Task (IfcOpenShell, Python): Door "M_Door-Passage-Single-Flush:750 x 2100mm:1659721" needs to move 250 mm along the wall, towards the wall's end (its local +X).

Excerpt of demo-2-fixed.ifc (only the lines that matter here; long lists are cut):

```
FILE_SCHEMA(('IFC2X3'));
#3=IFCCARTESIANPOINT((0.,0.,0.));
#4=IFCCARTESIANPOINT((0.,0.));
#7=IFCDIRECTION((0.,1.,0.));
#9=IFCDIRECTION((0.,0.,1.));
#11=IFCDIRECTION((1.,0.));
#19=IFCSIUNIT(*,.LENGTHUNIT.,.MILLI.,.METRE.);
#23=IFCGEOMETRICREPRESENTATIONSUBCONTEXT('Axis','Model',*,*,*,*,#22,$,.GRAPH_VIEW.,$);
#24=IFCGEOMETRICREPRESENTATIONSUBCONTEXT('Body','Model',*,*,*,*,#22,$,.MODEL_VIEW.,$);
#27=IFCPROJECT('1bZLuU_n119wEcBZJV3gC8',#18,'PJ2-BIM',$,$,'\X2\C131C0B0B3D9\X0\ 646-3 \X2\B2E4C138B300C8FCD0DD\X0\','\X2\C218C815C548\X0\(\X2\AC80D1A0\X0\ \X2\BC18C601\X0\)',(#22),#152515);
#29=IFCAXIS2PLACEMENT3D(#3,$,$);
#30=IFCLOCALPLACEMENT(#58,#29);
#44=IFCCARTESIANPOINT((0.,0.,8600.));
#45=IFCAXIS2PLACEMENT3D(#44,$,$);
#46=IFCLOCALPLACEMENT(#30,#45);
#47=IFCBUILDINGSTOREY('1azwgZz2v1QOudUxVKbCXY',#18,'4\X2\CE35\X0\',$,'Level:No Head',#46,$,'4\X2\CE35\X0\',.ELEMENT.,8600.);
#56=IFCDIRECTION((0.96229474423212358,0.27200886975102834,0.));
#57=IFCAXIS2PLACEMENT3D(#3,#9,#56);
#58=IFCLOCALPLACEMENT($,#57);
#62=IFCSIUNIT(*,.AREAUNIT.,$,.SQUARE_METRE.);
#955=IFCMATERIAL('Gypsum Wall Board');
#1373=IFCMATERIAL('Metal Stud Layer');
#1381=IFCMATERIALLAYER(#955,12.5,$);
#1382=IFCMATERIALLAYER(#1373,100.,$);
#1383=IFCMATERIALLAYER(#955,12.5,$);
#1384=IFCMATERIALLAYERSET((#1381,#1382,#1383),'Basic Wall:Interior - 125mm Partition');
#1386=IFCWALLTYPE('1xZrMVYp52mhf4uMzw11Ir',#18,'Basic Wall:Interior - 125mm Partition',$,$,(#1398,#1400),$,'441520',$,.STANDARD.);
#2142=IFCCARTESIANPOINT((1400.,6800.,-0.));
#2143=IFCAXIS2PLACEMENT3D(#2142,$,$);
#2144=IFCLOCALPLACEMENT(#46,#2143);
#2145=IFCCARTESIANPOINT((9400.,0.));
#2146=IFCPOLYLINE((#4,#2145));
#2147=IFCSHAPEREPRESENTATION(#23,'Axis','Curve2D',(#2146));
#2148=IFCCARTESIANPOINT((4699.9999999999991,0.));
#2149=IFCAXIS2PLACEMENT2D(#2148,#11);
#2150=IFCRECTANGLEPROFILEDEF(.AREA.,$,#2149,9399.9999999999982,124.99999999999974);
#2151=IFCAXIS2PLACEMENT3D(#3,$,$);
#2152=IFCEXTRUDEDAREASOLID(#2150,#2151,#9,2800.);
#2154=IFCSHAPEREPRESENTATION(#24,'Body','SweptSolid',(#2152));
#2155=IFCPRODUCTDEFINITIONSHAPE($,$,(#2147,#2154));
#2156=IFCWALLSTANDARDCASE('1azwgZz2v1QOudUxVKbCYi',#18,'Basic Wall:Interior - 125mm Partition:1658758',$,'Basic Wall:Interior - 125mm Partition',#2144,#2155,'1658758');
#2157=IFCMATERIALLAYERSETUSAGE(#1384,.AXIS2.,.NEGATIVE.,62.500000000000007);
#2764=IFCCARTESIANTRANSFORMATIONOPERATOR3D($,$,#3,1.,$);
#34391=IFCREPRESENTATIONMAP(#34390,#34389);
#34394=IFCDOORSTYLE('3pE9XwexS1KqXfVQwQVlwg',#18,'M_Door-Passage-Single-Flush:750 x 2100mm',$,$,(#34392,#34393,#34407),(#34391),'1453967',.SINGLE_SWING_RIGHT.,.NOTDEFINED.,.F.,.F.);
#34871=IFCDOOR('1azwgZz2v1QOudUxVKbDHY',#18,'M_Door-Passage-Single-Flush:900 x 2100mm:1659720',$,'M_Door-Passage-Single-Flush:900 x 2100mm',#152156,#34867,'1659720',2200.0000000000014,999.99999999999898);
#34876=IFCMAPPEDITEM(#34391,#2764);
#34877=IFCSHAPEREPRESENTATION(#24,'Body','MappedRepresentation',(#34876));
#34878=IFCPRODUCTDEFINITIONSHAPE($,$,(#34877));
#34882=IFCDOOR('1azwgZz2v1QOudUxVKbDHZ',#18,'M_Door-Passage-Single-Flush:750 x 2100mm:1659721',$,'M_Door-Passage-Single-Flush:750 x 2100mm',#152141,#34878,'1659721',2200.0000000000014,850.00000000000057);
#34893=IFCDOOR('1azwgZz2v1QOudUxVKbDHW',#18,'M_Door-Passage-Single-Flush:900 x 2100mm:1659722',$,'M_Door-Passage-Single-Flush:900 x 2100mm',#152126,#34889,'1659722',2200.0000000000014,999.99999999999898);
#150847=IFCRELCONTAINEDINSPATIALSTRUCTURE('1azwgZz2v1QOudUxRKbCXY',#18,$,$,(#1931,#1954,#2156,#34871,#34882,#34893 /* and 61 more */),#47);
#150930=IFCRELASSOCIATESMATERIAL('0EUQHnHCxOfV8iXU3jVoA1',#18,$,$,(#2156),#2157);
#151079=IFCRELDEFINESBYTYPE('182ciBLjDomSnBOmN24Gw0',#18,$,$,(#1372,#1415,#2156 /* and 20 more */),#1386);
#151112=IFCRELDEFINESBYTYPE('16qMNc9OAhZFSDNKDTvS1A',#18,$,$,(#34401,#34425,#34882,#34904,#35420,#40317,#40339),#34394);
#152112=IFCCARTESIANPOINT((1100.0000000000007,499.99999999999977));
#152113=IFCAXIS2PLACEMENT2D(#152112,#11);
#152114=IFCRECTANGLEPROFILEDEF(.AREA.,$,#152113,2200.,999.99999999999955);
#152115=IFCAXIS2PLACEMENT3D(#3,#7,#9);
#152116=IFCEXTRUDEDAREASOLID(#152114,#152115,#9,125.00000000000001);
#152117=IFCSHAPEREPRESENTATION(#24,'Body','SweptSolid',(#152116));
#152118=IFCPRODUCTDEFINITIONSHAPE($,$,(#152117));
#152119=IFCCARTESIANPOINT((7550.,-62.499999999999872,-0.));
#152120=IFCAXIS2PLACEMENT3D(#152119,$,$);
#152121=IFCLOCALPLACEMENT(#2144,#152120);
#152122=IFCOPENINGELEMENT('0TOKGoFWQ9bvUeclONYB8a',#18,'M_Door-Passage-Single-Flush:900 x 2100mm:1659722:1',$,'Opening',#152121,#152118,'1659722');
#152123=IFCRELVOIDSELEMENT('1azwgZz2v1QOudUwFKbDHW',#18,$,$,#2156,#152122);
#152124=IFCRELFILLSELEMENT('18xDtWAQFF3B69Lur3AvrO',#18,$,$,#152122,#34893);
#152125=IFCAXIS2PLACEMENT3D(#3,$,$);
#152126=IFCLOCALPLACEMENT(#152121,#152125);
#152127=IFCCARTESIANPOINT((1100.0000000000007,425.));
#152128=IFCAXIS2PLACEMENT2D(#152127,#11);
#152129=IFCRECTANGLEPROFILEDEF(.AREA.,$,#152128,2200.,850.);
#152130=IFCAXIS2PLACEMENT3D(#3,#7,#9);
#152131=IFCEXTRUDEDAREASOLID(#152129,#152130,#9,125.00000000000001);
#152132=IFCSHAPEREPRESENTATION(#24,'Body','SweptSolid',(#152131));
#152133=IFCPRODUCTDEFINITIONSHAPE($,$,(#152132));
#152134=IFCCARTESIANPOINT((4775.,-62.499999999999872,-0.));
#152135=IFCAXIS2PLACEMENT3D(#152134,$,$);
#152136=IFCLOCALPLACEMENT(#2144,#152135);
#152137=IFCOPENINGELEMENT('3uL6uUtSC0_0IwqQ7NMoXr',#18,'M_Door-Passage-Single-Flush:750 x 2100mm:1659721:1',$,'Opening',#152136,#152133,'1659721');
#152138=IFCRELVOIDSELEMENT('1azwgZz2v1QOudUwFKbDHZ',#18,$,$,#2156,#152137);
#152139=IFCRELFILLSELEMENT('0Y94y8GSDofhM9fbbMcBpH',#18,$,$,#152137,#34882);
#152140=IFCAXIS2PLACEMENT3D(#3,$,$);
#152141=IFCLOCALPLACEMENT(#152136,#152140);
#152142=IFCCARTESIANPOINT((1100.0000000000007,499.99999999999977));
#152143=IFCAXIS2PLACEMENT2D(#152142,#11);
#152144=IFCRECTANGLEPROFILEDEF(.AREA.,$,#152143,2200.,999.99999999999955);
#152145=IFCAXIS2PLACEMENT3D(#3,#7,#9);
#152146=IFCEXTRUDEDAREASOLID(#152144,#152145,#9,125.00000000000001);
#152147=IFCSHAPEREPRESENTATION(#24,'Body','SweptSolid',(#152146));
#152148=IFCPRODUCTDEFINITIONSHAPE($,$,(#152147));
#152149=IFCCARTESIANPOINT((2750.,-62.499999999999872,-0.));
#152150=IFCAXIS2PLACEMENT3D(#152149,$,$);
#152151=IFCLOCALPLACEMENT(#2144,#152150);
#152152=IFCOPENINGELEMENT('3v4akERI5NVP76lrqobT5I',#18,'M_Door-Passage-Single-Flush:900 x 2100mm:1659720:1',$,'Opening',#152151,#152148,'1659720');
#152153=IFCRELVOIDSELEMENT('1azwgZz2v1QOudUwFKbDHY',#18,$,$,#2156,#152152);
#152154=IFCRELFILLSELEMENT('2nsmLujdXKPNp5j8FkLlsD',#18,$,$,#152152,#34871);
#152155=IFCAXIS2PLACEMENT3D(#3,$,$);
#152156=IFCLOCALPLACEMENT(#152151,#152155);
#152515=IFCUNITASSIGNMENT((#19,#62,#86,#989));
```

```python
import ifcopenshell
import ifcopenshell.api.geometry
import ifcopenshell.util.placement
import ifcopenshell.util.unit

model = ifcopenshell.open("demo-2-fixed.ifc")
unit_scale = ifcopenshell.util.unit.calculate_unit_scale(model)

door = model.by_guid("1azwgZz2v1QOudUxVKbDHZ")
opening = door.FillsVoids[0].RelatingOpeningElement
wall = opening.VoidsElements[0].RelatingBuildingElement

wall_matrix = ifcopenshell.util.placement.get_local_placement(wall.ObjectPlacement)
shift = wall_matrix[:3, 0] * 0.25 / unit_scale
before = ifcopenshell.util.placement.get_local_placement(door.ObjectPlacement)[:3, 3].copy()

# The door is placed relative to its opening, so it follows when the opening moves.
matrix = ifcopenshell.util.placement.get_local_placement(opening.ObjectPlacement)
matrix[:3, 3] += shift
ifcopenshell.api.geometry.edit_object_placement(
    model, product=opening, matrix=matrix, is_si=False, should_transform_children=True
)

after = ifcopenshell.util.placement.get_local_placement(door.ObjectPlacement)[:3, 3]
print("door moved by", (after - before).round(3) + 0.0)

model.write("demo-2-fixed-out.ifc")
```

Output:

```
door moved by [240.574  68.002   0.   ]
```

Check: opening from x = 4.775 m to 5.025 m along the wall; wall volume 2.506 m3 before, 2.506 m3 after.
